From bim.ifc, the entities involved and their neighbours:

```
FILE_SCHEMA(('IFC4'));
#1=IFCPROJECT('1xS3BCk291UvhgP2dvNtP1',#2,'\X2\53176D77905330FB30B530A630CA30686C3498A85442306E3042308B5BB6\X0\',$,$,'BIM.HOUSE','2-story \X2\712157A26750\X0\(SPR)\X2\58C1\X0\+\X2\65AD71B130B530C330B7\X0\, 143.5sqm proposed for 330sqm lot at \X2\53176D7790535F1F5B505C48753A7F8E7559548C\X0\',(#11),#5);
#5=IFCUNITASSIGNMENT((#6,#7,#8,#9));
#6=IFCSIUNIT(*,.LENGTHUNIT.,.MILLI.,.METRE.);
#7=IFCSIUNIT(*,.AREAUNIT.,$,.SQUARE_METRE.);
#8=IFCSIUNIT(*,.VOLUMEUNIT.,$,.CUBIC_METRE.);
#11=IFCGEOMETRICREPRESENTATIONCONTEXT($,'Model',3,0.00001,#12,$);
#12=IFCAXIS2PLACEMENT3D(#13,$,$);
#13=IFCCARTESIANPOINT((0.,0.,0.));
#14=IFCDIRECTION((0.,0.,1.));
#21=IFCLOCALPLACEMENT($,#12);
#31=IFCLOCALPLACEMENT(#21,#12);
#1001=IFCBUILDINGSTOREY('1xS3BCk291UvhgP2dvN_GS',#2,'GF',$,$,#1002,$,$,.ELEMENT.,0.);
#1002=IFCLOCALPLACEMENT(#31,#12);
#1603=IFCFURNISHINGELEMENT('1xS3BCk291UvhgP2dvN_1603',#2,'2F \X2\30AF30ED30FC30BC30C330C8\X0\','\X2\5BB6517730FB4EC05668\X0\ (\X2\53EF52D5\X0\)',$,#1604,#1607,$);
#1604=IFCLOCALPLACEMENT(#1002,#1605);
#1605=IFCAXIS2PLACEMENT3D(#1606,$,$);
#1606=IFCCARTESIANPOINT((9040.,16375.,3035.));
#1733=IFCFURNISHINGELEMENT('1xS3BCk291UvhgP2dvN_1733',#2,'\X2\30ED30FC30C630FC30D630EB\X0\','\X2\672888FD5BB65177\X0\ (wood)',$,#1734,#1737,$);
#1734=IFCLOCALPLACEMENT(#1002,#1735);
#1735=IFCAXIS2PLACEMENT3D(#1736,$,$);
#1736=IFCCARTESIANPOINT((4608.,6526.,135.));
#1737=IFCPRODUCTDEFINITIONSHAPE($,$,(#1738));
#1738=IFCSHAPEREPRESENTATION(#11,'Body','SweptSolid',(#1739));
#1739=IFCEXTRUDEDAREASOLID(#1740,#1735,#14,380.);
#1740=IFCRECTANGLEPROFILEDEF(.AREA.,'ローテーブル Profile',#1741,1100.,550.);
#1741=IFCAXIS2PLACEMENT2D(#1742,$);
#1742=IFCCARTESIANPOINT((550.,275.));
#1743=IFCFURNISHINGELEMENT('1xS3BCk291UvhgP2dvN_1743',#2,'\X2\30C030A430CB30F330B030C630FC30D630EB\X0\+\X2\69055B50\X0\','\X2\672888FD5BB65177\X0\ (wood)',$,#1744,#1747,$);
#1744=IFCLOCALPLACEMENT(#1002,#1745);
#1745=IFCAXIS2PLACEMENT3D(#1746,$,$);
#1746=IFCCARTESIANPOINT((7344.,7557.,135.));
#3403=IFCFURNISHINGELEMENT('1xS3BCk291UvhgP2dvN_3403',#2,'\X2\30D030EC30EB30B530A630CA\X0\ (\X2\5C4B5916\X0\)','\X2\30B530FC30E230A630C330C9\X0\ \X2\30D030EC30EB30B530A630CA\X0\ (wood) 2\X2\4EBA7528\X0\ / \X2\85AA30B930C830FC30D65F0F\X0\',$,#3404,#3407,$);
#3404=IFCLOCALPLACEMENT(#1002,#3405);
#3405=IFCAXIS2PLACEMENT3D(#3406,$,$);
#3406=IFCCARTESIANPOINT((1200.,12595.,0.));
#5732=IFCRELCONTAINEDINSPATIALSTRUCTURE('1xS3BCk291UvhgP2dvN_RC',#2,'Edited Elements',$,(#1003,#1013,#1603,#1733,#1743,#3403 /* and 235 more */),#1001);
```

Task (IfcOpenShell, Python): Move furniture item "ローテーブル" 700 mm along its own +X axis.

```python
import ifcopenshell
import ifcopenshell.api.geometry
import ifcopenshell.util.placement
import ifcopenshell.util.unit

model = ifcopenshell.open("bim.ifc")
unit_scale = ifcopenshell.util.unit.calculate_unit_scale(model)

item = model.by_guid("1xS3BCk291UvhgP2dvN_1733")
matrix = ifcopenshell.util.placement.get_local_placement(item.ObjectPlacement)
matrix[:3, 3] += matrix[:3, 0] * 0.7 / unit_scale
ifcopenshell.api.geometry.edit_object_placement(model, product=item, matrix=matrix, is_si=False)

print(ifcopenshell.util.placement.get_local_placement(item.ObjectPlacement).round(3) + 0.0)

model.write("bim_rev.ifc")
```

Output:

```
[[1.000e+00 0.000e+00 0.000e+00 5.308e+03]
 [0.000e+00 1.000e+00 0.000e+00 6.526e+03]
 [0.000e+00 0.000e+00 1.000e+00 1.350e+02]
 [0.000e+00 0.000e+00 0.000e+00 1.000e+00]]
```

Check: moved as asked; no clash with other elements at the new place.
